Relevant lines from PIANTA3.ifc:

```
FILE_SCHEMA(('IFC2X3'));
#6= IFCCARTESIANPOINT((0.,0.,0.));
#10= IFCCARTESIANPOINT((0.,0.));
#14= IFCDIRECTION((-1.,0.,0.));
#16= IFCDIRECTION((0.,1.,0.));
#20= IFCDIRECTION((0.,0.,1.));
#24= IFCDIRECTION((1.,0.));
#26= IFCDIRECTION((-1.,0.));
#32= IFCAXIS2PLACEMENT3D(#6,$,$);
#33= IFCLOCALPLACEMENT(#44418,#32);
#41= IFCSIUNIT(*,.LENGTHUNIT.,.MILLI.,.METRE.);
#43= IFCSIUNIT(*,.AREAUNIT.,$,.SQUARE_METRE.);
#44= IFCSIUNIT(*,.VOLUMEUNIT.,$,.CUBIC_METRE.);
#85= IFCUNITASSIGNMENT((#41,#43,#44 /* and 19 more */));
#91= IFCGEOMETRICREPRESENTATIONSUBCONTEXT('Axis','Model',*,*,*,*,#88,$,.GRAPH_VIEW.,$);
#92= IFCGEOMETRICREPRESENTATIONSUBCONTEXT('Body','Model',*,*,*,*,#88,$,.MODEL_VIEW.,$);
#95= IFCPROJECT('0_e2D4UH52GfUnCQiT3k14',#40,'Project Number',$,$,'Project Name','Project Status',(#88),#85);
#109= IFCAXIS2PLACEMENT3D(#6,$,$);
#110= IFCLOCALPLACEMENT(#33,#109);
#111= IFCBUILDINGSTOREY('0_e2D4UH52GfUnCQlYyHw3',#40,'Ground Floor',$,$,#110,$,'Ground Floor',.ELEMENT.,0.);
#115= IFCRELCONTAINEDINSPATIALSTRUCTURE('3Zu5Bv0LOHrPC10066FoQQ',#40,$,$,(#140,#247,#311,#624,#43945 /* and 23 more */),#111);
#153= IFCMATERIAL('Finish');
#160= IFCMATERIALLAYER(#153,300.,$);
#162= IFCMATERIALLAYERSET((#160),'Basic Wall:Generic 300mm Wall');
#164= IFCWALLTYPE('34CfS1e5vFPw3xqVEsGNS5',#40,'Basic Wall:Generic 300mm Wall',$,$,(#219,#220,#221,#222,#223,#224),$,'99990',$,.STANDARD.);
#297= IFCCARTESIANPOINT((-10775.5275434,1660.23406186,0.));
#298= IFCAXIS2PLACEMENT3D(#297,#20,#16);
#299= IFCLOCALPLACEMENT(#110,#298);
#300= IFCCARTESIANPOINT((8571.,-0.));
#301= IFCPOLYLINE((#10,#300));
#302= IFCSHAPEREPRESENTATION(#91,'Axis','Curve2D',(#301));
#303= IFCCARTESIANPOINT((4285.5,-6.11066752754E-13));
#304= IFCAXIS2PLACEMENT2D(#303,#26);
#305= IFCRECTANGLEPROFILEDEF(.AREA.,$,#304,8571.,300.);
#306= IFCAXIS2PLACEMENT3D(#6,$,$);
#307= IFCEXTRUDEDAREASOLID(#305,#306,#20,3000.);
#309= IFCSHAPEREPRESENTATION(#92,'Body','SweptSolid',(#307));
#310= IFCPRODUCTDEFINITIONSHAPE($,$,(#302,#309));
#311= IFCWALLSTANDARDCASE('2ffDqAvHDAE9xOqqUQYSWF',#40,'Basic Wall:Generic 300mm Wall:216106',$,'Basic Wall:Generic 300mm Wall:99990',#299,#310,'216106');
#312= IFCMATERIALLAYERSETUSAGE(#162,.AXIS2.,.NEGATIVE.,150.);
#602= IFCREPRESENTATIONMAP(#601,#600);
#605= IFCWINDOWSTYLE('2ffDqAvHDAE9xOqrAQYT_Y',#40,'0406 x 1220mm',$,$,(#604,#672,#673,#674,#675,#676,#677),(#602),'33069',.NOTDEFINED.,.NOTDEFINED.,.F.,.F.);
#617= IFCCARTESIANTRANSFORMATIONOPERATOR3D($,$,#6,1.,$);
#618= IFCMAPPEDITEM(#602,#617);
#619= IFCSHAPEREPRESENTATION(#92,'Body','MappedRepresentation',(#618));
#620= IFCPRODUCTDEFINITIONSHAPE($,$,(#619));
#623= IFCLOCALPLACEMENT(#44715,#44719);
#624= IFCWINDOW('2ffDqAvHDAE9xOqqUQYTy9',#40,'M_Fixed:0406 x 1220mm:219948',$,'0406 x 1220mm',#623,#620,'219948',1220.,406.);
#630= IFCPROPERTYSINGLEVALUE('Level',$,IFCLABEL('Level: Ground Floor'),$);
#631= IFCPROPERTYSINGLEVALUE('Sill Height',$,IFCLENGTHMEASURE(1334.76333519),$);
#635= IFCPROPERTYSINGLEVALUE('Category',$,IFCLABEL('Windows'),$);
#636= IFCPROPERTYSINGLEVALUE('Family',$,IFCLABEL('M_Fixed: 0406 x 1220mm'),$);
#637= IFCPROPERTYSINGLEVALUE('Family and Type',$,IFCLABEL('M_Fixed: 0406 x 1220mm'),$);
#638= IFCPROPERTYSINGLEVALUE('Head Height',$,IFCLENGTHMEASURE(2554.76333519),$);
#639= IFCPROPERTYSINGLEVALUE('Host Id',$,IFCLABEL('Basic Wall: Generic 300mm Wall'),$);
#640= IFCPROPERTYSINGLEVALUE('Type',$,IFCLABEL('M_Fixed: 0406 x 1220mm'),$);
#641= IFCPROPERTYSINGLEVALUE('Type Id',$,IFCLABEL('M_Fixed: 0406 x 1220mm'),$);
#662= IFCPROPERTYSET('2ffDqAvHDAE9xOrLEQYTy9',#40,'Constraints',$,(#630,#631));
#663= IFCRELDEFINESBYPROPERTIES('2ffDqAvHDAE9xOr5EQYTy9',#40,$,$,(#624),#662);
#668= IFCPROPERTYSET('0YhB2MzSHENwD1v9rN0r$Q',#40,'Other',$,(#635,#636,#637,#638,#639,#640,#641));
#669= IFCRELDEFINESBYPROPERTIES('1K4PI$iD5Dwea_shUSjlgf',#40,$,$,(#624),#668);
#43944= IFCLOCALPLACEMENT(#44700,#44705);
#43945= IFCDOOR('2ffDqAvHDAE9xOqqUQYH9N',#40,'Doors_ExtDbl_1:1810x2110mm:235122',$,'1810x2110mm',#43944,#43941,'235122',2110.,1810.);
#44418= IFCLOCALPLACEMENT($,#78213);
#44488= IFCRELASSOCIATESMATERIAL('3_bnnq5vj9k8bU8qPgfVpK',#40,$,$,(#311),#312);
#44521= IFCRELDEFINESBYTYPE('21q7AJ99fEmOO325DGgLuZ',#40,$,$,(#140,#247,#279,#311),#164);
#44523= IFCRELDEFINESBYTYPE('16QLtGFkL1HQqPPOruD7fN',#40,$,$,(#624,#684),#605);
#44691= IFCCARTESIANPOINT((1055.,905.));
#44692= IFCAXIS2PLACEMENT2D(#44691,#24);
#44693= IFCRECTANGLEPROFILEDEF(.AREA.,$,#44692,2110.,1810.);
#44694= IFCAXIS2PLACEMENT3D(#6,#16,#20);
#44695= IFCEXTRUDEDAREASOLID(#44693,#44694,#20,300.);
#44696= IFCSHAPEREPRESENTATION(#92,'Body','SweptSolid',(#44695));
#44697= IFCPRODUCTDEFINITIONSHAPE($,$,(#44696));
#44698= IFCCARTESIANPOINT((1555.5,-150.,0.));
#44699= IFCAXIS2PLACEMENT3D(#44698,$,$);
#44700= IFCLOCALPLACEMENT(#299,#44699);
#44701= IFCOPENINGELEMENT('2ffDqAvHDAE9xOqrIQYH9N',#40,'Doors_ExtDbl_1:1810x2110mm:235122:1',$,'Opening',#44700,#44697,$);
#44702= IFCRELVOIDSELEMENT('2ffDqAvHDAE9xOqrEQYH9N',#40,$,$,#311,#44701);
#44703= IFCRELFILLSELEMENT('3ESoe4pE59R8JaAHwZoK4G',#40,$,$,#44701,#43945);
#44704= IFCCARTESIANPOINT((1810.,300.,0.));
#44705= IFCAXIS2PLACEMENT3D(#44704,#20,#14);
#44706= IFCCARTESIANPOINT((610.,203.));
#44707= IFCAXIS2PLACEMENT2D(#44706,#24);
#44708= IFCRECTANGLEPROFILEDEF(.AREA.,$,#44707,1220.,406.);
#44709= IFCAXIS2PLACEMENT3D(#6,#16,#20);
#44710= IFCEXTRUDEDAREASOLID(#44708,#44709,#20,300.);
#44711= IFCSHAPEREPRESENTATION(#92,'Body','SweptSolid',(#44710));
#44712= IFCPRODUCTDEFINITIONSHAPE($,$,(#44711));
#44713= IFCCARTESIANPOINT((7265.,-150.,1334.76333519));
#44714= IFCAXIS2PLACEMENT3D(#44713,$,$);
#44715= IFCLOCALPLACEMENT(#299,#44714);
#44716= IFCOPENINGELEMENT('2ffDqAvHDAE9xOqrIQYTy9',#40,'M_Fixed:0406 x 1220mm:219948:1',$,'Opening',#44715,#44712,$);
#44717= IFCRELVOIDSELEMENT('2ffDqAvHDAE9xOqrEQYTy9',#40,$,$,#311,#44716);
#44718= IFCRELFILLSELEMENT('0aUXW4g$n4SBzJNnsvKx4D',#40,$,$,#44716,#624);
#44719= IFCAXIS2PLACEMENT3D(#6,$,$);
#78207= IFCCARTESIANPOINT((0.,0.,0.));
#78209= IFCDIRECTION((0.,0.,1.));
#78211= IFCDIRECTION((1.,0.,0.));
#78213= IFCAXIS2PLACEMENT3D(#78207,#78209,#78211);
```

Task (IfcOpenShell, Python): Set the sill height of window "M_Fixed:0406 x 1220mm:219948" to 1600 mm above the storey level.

```python
import numpy as np
import ifcopenshell
import ifcopenshell.api.geometry
import ifcopenshell.api.pset
import ifcopenshell.geom
import ifcopenshell.util.element
import ifcopenshell.util.placement
import ifcopenshell.util.shape
import ifcopenshell.util.unit

model = ifcopenshell.open("PIANTA3.ifc")
unit_scale = ifcopenshell.util.unit.calculate_unit_scale(model)

window = model.by_guid("2ffDqAvHDAE9xOqqUQYTy9")
opening = window.FillsVoids[0].RelatingOpeningElement
storey = ifcopenshell.util.element.get_container(window, ifc_class="IfcBuildingStorey")
level = ifcopenshell.util.placement.get_local_placement(storey.ObjectPlacement)[2, 3]

# The opening's origin need not be at the sill, so measure its lowest point.
shape = ifcopenshell.geom.create_shape(ifcopenshell.geom.settings(), opening)
bottom = ifcopenshell.util.shape.get_shape_bottom_elevation(shape, shape.geometry) / unit_scale
dz = level + 1.6 / unit_scale - bottom

shift = np.array([0.0, 0.0, dz])
# The window is placed relative to its opening, so it follows when the opening moves.
matrix = ifcopenshell.util.placement.get_local_placement(opening.ObjectPlacement)
matrix[:3, 3] += shift
ifcopenshell.api.geometry.edit_object_placement(
    model, product=opening, matrix=matrix, is_si=False, should_transform_children=True
)

# Keep the stored heights in step.
pset = model.by_id(ifcopenshell.util.element.get_pset(window, "Constraints", should_inherit=False)["id"])
ifcopenshell.api.pset.edit_pset(model, pset=pset, properties={
    "Sill Height": model.create_entity("IfcLengthMeasure", ifcopenshell.util.element.get_pset(window, "Constraints", "Sill Height") + dz),
})
pset = model.by_id(ifcopenshell.util.element.get_pset(window, "Other", should_inherit=False)["id"])
ifcopenshell.api.pset.edit_pset(model, pset=pset, properties={
    "Head Height": model.create_entity("IfcLengthMeasure", ifcopenshell.util.element.get_pset(window, "Other", "Head Height") + dz),
})

print(f"moved by {dz * unit_scale:+.3f} m")

model.write("PIANTA3_rev.ifc")
```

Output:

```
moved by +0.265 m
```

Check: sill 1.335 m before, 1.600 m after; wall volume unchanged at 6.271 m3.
